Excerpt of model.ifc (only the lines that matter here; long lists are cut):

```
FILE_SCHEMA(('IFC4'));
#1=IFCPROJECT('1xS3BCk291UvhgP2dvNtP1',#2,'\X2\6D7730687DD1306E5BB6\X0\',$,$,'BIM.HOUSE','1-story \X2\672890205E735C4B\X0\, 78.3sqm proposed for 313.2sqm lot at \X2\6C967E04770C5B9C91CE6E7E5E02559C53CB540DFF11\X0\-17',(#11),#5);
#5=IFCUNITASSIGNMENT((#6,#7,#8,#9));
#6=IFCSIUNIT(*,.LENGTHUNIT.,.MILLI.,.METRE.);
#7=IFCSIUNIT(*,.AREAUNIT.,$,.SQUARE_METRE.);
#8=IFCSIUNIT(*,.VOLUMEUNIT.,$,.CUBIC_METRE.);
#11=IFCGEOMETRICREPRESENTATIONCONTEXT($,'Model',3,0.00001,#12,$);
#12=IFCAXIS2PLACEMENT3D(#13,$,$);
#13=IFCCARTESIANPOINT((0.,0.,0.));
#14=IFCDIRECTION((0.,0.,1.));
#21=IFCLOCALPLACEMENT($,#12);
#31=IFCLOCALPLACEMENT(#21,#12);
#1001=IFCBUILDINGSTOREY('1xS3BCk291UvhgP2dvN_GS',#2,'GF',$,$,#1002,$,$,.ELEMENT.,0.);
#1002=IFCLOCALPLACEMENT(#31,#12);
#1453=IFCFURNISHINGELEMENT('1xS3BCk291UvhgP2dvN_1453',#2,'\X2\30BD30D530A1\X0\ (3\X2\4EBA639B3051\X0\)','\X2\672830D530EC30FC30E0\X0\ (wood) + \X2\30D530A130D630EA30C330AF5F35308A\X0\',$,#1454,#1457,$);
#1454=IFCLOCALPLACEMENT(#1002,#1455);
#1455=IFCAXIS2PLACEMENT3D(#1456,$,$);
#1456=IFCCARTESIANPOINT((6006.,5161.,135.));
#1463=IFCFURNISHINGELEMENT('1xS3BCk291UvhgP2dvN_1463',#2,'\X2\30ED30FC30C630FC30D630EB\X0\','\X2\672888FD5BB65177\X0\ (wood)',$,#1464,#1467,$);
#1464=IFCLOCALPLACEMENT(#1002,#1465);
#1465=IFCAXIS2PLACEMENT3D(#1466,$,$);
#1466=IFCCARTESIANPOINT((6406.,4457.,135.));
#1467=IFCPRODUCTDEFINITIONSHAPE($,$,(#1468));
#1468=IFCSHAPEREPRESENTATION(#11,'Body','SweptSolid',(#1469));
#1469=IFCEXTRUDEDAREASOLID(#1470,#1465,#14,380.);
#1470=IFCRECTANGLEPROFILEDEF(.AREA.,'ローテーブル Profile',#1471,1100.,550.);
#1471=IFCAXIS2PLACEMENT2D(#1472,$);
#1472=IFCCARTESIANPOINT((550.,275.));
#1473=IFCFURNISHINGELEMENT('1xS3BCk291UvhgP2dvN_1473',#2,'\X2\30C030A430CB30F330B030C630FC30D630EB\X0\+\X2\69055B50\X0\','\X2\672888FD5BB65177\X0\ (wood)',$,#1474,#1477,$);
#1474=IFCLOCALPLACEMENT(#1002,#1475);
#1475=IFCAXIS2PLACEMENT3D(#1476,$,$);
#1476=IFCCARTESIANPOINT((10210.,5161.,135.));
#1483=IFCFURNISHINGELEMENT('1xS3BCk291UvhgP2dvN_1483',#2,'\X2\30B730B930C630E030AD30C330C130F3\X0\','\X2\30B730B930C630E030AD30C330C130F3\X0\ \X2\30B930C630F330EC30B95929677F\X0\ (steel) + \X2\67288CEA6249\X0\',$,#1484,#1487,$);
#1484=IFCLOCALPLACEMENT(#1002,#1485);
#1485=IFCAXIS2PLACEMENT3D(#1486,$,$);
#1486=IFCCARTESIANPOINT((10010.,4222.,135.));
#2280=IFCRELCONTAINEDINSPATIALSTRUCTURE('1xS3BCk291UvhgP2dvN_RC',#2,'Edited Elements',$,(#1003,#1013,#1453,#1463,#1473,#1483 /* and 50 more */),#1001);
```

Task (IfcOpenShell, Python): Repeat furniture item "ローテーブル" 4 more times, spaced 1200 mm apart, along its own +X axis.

```python
import ifcopenshell
import ifcopenshell.api.geometry
import ifcopenshell.api.root
import ifcopenshell.util.element
import ifcopenshell.util.placement
import ifcopenshell.util.unit

model = ifcopenshell.open("model.ifc")
unit_scale = ifcopenshell.util.unit.calculate_unit_scale(model)


def reuse_history(source, copy):
    """copy_class also copies each property set's owner history, people and application; keep the originals."""
    for rel in copy.IsDefinedBy:
        if rel.is_a("IfcRelDefinesByProperties") and (history := rel.RelatingPropertyDefinition.OwnerHistory):
            rel.RelatingPropertyDefinition.OwnerHistory = source.OwnerHistory
            ifcopenshell.util.element.remove_deep2(model, history)


source = model.by_guid("1xS3BCk291UvhgP2dvN_1463")
base = ifcopenshell.util.placement.get_local_placement(source.ObjectPlacement)
step = base[:3, 0] * 1.2 / unit_scale

for i in range(1, 5):
    copy = ifcopenshell.api.root.copy_class(model, product=source)
    copy.Representation = ifcopenshell.util.element.copy_deep(
        model, source.Representation, exclude=["IfcGeometricRepresentationContext", "IfcRepresentationMap"]
    )
    reuse_history(source, copy)
    matrix = base.copy()
    matrix[:3, 3] += i * step
    print("added at", matrix[:3, 3].round(3) + 0.0)
    ifcopenshell.api.geometry.edit_object_placement(model, product=copy, matrix=matrix, is_si=False)

model.write("model_v2.ifc")
```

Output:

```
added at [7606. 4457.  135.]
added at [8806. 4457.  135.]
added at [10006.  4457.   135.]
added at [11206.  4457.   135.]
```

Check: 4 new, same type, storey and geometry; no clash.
